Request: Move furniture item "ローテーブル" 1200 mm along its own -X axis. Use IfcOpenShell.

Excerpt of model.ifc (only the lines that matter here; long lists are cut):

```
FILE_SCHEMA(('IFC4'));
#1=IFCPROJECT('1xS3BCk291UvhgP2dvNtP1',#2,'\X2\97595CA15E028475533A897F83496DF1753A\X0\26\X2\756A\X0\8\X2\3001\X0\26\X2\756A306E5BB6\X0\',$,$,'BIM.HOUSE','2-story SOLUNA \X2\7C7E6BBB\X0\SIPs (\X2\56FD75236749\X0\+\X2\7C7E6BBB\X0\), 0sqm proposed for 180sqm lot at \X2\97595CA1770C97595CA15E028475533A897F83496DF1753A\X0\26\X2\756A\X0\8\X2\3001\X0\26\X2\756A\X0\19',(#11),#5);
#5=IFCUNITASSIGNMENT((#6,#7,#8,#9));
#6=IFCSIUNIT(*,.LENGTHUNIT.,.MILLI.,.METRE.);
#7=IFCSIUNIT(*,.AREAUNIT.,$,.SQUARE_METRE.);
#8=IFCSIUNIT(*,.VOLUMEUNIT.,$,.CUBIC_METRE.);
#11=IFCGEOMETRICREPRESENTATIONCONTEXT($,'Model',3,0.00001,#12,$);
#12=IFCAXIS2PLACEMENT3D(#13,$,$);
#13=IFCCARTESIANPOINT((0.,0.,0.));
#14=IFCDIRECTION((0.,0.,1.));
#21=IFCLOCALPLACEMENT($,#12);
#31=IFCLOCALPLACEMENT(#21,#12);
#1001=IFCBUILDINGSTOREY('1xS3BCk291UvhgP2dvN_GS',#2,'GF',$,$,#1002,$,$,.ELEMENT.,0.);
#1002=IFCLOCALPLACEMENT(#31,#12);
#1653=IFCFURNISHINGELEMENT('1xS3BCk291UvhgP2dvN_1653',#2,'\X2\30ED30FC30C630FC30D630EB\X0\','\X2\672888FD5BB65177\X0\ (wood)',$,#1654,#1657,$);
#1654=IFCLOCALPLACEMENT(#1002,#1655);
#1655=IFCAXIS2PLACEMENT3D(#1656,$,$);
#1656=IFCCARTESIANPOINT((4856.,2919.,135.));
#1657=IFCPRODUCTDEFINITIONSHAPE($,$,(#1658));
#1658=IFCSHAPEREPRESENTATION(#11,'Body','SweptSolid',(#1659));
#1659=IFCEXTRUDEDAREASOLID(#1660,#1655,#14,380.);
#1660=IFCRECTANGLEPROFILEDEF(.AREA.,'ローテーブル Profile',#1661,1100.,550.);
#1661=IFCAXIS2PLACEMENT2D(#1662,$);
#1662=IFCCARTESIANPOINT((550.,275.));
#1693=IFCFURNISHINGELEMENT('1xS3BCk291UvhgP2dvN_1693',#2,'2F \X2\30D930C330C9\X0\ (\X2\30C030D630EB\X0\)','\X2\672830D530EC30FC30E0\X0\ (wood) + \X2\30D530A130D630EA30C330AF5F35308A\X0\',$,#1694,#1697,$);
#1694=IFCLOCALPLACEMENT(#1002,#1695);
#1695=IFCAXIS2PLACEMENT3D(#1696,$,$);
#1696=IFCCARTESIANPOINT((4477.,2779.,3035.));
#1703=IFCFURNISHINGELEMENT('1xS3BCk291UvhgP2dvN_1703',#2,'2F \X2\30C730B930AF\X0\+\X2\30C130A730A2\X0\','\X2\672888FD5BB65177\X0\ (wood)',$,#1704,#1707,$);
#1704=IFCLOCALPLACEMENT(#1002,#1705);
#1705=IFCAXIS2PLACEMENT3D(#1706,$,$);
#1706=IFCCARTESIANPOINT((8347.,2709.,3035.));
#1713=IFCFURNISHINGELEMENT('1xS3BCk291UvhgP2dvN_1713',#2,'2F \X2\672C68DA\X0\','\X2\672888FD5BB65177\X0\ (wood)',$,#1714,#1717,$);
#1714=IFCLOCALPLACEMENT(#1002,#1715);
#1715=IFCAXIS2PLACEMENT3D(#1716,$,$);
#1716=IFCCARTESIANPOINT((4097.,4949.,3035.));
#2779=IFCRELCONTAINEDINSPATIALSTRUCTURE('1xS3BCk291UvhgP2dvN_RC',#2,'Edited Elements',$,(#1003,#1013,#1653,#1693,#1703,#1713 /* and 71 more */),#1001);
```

```python
import ifcopenshell
import ifcopenshell.api.geometry
import ifcopenshell.util.placement

model = ifcopenshell.open("model.ifc")

item = model.by_guid("1xS3BCk291UvhgP2dvN_1653")
matrix = ifcopenshell.util.placement.get_local_placement(item.ObjectPlacement)
matrix[:3, 3] -= matrix[:3, 0] * 1200.0
ifcopenshell.api.geometry.edit_object_placement(model, product=item, matrix=matrix, is_si=False)

print(ifcopenshell.util.placement.get_local_placement(item.ObjectPlacement).round(3) + 0.0)

model.write("model_updated.ifc")
```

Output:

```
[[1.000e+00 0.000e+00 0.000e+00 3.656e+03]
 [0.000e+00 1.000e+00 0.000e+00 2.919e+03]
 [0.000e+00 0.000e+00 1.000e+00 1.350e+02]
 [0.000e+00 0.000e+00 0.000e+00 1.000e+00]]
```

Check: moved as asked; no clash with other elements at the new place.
